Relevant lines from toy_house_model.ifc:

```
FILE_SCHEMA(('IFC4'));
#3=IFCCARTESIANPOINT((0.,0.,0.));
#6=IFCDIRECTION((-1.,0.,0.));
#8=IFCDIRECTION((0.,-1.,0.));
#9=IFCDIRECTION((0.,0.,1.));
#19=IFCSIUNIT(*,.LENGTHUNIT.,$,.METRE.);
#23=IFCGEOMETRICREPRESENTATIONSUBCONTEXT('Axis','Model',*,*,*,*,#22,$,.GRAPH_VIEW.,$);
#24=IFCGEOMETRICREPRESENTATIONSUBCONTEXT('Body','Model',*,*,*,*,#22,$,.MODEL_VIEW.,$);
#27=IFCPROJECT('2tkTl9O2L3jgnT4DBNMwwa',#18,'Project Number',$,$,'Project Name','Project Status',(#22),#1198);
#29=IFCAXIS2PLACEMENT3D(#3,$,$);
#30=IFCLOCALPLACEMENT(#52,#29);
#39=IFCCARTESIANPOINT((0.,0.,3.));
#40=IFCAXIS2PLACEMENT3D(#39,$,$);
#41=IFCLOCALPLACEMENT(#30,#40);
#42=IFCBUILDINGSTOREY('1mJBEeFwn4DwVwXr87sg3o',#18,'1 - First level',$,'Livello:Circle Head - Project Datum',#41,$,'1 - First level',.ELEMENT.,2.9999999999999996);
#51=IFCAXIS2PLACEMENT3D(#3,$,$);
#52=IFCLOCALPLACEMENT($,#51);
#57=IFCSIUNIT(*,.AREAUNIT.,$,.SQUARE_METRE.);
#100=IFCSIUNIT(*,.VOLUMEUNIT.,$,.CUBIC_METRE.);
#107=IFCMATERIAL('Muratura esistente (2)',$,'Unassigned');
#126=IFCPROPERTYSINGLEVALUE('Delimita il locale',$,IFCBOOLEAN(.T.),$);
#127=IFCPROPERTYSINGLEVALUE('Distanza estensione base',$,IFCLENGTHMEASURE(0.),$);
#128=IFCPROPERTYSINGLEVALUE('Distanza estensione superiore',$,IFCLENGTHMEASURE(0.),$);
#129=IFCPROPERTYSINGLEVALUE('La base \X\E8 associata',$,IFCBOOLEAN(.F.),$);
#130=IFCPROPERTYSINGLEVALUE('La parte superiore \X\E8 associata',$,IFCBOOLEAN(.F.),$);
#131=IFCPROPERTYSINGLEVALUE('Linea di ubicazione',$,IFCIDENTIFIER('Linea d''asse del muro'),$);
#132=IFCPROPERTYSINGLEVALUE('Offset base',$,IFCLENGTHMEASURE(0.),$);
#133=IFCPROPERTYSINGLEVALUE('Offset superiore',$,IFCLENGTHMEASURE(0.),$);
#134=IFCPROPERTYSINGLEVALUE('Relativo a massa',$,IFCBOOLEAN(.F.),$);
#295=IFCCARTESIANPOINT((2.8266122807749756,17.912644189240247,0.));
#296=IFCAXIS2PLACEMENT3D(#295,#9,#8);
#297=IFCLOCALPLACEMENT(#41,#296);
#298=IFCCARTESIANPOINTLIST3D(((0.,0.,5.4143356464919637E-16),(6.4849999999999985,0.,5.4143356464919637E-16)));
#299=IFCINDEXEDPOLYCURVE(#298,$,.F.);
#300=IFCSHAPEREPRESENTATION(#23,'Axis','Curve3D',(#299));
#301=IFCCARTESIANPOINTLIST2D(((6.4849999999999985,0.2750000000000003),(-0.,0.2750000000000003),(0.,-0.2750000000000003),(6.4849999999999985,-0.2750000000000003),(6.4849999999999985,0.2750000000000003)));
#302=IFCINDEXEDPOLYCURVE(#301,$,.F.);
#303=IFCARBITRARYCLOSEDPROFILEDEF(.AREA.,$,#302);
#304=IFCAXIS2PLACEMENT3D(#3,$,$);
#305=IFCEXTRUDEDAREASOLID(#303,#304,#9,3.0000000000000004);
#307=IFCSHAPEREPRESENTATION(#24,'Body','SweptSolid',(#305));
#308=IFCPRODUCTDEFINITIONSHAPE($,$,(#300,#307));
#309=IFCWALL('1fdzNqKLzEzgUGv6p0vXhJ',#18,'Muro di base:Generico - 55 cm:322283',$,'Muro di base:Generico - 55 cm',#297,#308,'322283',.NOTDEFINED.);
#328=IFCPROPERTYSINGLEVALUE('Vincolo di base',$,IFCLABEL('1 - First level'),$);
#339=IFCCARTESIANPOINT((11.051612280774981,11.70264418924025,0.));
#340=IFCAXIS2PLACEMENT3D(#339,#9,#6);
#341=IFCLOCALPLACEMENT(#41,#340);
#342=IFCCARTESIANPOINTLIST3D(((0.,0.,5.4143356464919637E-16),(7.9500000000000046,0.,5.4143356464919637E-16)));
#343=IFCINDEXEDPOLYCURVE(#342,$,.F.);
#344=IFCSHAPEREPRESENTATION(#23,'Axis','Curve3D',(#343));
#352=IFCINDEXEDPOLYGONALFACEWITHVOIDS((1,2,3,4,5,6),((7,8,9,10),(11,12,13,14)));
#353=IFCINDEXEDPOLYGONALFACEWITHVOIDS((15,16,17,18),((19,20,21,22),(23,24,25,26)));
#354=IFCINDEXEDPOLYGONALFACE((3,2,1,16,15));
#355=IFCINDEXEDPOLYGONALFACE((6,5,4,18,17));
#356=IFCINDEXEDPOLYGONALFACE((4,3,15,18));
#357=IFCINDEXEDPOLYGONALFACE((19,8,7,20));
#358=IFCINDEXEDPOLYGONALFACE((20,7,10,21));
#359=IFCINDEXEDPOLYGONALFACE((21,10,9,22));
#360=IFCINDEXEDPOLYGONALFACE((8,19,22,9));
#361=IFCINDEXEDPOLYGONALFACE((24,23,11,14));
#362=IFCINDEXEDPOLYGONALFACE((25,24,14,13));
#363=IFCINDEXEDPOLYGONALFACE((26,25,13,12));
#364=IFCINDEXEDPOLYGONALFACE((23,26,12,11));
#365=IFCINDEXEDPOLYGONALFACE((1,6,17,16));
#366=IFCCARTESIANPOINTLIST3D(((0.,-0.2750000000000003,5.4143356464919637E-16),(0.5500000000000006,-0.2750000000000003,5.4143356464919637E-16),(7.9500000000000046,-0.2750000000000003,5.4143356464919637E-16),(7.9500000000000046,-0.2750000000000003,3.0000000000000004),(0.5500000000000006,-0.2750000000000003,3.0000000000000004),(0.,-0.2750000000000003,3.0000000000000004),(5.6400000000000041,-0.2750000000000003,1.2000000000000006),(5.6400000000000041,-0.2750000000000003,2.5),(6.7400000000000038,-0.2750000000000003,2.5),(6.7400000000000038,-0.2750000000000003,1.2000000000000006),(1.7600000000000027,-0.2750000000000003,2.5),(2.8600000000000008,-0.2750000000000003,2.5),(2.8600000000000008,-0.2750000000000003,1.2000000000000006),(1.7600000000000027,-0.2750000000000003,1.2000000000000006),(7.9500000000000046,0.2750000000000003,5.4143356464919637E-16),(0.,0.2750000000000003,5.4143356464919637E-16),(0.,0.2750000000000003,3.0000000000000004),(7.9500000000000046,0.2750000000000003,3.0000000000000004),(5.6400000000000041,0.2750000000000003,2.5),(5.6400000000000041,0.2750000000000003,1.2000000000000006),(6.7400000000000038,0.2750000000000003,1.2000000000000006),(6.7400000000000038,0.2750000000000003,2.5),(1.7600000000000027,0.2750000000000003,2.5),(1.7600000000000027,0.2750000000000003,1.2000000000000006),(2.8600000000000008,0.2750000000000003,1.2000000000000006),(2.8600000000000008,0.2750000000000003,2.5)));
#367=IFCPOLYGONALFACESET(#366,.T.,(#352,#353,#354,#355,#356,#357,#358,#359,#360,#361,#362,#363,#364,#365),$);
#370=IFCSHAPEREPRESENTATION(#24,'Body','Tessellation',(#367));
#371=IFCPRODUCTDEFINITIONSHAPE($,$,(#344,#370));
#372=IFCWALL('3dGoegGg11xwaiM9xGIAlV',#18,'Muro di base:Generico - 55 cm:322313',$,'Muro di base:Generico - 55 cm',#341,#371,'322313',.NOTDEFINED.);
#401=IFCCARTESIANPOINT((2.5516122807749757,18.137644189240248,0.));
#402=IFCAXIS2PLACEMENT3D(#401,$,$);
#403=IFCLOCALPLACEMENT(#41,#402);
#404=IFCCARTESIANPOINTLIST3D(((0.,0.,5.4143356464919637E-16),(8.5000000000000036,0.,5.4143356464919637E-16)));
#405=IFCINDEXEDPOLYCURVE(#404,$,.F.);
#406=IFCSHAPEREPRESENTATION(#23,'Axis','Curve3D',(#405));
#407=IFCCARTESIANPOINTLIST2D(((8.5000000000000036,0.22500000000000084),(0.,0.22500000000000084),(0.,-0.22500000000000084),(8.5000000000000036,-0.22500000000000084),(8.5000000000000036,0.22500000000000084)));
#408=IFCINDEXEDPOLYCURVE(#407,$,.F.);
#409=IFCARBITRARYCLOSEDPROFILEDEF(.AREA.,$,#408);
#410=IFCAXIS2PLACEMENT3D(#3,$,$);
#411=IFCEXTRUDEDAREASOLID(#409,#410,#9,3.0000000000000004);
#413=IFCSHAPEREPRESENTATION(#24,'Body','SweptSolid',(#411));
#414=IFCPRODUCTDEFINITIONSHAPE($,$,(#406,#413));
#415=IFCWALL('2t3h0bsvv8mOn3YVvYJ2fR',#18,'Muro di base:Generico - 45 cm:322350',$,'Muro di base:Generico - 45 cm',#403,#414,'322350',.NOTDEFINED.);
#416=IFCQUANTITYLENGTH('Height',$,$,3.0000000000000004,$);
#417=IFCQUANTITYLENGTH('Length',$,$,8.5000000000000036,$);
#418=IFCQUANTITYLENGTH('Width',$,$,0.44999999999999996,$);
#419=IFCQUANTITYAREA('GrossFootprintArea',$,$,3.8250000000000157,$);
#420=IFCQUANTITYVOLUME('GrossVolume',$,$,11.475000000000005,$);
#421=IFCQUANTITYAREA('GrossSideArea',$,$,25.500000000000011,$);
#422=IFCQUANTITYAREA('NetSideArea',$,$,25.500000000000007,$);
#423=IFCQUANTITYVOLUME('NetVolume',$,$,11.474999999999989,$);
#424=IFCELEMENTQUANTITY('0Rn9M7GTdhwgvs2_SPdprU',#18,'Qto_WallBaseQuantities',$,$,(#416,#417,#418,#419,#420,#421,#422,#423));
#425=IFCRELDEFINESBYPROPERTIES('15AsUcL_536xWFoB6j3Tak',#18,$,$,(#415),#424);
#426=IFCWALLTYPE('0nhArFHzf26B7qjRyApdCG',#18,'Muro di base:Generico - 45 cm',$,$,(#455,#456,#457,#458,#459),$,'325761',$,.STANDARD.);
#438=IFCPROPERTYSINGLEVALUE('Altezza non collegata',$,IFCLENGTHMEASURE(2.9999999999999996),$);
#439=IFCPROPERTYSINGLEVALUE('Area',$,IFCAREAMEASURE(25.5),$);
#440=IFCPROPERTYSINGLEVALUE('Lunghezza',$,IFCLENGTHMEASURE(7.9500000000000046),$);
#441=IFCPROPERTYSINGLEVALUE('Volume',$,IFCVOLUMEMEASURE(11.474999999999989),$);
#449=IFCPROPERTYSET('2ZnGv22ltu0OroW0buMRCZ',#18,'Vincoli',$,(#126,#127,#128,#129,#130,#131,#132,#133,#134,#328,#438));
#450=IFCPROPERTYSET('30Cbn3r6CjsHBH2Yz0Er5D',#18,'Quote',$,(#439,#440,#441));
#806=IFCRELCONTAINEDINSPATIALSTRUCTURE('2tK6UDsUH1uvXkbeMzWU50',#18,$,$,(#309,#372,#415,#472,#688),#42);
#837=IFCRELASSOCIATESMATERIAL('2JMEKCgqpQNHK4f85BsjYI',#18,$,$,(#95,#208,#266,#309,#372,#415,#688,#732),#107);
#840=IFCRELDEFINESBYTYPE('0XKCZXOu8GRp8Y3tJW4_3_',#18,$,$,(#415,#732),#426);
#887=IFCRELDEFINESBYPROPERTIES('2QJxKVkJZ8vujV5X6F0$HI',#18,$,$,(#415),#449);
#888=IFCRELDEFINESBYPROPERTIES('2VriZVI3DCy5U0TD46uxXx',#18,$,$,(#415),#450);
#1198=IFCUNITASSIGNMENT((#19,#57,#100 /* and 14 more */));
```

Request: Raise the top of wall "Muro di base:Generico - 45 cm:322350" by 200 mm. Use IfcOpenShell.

```python
import ifcopenshell
import ifcopenshell.api.pset
import ifcopenshell.geom
import ifcopenshell.util.element
import ifcopenshell.util.representation
import ifcopenshell.util.shape
import ifcopenshell.util.unit

model = ifcopenshell.open("toy_house_model.ifc")
unit_scale = ifcopenshell.util.unit.calculate_unit_scale(model)
area_scale = ifcopenshell.util.unit.calculate_unit_scale(model, "AREAUNIT")
volume_scale = ifcopenshell.util.unit.calculate_unit_scale(model, "VOLUMEUNIT")
settings = ifcopenshell.geom.settings()


def volume(element):
    """Net volume in cubic metres, openings subtracted."""
    shape = ifcopenshell.geom.create_shape(settings, element)
    return ifcopenshell.util.shape.get_volume(shape.geometry)


wall = model.by_guid("2t3h0bsvv8mOn3YVvYJ2fR")
before = volume(wall)

body = ifcopenshell.util.representation.get_representation(wall, "Model", "Body")
solid = body.Items[0]
old_height = solid.Depth
solid.Depth += 0.2 / unit_scale
after = volume(wall)
thickness = 0.45  # wall thickness in metres

# Update the stored height, areas and volumes.
qto = model.by_id(ifcopenshell.util.element.get_pset(wall, "Qto_WallBaseQuantities", should_inherit=False)["id"])
ifcopenshell.api.pset.edit_qto(model, qto=qto, properties={
    "Height": solid.Depth,
    "GrossVolume": ifcopenshell.util.element.get_pset(wall, "Qto_WallBaseQuantities", "GrossVolume") * solid.Depth / old_height,
    "GrossSideArea": ifcopenshell.util.element.get_pset(wall, "Qto_WallBaseQuantities", "GrossSideArea") * solid.Depth / old_height,
    "NetSideArea": after / thickness / area_scale,
    "NetVolume": after / volume_scale,
})
pset = model.by_id(ifcopenshell.util.element.get_pset(wall, "Vincoli", should_inherit=False)["id"])
ifcopenshell.api.pset.edit_pset(model, pset=pset, properties={
    "Altezza non collegata": model.create_entity("IfcLengthMeasure", solid.Depth),
})
pset = model.by_id(ifcopenshell.util.element.get_pset(wall, "Quote", should_inherit=False)["id"])
ifcopenshell.api.pset.edit_pset(model, pset=pset, properties={
    "Area": model.create_entity("IfcAreaMeasure", after / thickness / area_scale),
    "Volume": model.create_entity("IfcVolumeMeasure", after / volume_scale),
})

print(f"height {old_height:g} -> {solid.Depth:g}, volume {before:.3f} -> {after:.3f} m3")

model.write("toy_house_model-out.ifc")
```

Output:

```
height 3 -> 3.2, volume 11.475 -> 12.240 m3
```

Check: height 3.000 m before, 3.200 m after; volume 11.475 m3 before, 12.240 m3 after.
